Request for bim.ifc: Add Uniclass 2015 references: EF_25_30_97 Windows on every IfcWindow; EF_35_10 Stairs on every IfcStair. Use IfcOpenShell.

First a look at what the model holds.

```python
import ifcopenshell

model = ifcopenshell.open("bim.ifc")
print(model.schema)
print("classifications:", [c.Name for c in model.by_type("IfcClassification")])
for ifc_class in ("IfcDoor", "IfcRoof", "IfcStair", "IfcWall", "IfcWindow"):
    print(ifc_class, len(model.by_type(ifc_class)))
```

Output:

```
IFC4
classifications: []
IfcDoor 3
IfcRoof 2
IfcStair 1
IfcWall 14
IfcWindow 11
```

```python
import ifcopenshell
import ifcopenshell.api.classification

model = ifcopenshell.open("bim.ifc")

system = ifcopenshell.api.classification.add_classification(model, classification="Uniclass 2015")

codes = {
    "IfcWindow": ("EF_25_30_97", "Windows"),
    "IfcStair": ("EF_35_10", "Stairs"),
}
for ifc_class, (code, name) in codes.items():
    products = model.by_type(ifc_class)
    ifcopenshell.api.classification.add_reference(
        model, products=products, classification=system, identification=code, name=name
    )
    print(code, len(products))

model.write("bim_v2.ifc")
```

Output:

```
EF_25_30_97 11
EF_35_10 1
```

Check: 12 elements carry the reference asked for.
